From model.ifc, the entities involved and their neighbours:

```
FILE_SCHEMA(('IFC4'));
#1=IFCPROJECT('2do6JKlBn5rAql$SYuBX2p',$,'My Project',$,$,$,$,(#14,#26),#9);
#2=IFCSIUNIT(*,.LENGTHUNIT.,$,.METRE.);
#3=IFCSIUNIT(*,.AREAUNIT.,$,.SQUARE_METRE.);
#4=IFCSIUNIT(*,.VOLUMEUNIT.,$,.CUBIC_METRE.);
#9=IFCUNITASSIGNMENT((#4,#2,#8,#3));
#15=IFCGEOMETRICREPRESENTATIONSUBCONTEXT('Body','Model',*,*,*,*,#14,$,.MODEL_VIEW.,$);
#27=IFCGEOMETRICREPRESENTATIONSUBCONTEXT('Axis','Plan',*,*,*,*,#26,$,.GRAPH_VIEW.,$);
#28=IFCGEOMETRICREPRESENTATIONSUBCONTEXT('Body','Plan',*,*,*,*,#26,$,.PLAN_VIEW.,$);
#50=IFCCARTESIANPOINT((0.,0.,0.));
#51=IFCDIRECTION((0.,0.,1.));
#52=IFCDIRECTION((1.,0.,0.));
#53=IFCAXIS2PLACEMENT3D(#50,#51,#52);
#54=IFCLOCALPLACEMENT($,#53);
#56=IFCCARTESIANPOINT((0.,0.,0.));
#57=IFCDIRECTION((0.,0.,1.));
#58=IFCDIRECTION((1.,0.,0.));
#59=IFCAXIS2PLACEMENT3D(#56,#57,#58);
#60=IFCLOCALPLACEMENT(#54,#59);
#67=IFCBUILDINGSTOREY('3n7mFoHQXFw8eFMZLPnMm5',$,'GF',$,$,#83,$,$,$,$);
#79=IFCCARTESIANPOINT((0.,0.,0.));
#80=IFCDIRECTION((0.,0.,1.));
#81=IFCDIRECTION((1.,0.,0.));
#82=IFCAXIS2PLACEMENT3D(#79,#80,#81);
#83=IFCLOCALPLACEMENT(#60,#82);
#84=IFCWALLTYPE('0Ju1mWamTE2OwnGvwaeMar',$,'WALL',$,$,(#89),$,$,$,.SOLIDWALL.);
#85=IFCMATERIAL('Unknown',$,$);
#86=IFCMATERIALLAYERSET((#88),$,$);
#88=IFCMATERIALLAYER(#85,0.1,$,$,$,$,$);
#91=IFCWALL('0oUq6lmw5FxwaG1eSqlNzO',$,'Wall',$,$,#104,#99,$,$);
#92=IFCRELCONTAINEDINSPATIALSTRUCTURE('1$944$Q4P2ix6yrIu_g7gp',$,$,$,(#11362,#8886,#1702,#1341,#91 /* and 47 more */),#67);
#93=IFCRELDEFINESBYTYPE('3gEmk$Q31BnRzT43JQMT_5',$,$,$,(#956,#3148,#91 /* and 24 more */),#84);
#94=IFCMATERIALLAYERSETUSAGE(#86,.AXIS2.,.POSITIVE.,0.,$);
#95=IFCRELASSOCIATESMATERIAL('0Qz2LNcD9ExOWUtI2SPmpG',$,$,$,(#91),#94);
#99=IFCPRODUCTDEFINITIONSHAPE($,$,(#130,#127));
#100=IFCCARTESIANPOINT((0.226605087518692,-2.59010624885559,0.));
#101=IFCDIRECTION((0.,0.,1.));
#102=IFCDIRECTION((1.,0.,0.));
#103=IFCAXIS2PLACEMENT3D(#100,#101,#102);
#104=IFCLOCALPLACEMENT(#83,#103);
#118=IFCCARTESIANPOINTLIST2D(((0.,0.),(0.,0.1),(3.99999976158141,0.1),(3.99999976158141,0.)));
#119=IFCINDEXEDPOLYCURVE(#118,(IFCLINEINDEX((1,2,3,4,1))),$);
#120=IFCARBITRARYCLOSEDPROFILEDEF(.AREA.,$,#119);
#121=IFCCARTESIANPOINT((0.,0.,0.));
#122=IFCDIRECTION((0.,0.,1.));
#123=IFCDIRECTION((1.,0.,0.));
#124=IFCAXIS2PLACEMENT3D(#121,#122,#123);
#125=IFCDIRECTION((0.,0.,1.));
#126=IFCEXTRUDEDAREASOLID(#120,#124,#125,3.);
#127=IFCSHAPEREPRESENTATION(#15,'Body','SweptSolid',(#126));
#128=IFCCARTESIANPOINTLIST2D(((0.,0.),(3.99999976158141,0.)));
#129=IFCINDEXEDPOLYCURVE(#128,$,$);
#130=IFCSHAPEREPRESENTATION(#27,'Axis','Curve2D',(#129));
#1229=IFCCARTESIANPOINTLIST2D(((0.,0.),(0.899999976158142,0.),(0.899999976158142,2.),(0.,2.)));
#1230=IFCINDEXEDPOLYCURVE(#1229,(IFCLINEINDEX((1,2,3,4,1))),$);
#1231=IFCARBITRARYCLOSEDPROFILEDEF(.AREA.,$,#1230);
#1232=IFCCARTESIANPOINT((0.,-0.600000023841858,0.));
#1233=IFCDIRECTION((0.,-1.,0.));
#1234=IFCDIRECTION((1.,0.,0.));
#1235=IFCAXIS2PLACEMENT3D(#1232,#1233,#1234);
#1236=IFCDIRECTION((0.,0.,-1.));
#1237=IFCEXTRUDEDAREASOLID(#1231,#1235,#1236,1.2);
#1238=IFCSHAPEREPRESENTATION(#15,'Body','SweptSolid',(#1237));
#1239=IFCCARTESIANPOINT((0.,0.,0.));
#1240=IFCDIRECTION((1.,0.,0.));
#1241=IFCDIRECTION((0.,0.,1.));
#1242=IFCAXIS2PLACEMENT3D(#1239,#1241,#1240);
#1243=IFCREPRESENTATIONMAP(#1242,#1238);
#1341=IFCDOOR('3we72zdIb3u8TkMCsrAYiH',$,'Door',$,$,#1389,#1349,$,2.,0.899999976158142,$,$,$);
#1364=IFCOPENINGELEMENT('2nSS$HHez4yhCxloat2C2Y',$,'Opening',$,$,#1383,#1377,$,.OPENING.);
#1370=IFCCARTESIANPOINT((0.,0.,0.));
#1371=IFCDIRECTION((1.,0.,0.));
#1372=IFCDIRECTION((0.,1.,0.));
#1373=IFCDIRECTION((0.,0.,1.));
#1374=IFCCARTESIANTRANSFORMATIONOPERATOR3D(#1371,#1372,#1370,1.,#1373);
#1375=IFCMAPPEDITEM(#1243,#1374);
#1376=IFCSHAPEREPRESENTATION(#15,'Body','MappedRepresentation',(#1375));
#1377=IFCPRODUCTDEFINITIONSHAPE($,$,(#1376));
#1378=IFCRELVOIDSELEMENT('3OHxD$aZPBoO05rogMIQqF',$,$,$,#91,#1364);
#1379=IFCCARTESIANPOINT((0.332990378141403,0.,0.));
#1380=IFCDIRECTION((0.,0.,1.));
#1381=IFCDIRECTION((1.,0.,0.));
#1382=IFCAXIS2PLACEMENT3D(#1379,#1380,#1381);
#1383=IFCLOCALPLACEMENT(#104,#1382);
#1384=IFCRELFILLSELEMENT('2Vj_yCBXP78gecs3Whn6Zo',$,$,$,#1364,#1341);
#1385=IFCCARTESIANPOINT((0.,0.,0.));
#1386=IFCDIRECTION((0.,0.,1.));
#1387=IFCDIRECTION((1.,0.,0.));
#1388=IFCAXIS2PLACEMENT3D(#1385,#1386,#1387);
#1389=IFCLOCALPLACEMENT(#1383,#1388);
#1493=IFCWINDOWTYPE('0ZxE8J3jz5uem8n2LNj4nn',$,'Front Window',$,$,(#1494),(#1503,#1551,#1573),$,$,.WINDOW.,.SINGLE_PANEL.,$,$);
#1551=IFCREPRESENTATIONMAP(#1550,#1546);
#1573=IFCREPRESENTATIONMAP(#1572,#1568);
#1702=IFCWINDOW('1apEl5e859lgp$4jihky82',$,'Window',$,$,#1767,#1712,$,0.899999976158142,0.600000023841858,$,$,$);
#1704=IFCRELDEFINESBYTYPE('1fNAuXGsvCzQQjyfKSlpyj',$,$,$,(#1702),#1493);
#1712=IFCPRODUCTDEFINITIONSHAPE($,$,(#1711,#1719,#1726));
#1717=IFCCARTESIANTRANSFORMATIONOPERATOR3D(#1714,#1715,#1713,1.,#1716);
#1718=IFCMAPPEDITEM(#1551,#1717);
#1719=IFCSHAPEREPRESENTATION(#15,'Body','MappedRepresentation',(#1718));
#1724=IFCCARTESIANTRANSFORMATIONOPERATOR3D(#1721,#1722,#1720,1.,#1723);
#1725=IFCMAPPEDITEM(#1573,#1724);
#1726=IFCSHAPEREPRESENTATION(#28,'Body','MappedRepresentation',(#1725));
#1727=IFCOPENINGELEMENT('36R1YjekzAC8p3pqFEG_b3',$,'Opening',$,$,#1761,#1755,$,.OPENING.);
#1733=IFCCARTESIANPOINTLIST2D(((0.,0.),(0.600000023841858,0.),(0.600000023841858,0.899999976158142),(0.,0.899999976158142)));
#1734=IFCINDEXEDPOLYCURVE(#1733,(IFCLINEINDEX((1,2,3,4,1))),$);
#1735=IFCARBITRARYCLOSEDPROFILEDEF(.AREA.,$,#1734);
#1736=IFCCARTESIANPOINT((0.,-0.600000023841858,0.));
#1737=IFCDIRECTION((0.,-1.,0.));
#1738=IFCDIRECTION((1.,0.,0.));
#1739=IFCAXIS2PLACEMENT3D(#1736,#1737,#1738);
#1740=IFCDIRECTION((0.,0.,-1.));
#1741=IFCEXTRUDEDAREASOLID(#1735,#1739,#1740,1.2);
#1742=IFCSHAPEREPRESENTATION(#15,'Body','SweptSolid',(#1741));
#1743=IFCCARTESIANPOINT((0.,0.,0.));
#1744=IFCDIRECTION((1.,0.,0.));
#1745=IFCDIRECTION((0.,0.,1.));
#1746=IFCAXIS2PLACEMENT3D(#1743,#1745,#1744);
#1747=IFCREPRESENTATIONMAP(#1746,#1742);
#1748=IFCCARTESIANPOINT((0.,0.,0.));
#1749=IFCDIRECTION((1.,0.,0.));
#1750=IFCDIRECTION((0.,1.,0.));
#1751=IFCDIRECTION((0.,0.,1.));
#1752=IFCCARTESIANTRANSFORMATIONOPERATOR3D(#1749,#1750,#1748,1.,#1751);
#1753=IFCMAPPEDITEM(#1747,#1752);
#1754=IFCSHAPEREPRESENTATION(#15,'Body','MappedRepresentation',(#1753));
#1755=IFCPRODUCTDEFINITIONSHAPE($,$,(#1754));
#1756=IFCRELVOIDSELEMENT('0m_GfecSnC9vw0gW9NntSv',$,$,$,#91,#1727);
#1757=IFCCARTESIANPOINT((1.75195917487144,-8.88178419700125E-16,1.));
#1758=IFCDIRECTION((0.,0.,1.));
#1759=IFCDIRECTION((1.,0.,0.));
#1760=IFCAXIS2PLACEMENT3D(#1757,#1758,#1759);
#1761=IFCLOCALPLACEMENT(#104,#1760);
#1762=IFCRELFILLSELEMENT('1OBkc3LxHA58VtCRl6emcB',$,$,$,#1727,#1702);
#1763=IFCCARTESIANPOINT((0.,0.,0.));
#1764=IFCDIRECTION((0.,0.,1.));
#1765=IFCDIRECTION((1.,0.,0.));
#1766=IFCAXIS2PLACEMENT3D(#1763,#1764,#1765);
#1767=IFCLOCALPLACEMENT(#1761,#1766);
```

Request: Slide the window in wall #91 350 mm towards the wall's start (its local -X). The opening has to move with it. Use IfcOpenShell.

```python
import ifcopenshell
import ifcopenshell.api.geometry
import ifcopenshell.util.placement
import ifcopenshell.util.unit

model = ifcopenshell.open("model.ifc")
unit_scale = ifcopenshell.util.unit.calculate_unit_scale(model)

window = model.by_guid("1apEl5e859lgp$4jihky82")
opening = window.FillsVoids[0].RelatingOpeningElement
wall = opening.VoidsElements[0].RelatingBuildingElement

wall_matrix = ifcopenshell.util.placement.get_local_placement(wall.ObjectPlacement)
shift = wall_matrix[:3, 0] * -0.35 / unit_scale
before = ifcopenshell.util.placement.get_local_placement(window.ObjectPlacement)[:3, 3].copy()

# The window is placed relative to its opening, so it follows when the opening moves.
matrix = ifcopenshell.util.placement.get_local_placement(opening.ObjectPlacement)
matrix[:3, 3] += shift
ifcopenshell.api.geometry.edit_object_placement(
    model, product=opening, matrix=matrix, is_si=False, should_transform_children=True
)

after = ifcopenshell.util.placement.get_local_placement(window.ObjectPlacement)[:3, 3]
print("window moved by", (after - before).round(3) + 0.0)

model.write("model_updated.ifc")
```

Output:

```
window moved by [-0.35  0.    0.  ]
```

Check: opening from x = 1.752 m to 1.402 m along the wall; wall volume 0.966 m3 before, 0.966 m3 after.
